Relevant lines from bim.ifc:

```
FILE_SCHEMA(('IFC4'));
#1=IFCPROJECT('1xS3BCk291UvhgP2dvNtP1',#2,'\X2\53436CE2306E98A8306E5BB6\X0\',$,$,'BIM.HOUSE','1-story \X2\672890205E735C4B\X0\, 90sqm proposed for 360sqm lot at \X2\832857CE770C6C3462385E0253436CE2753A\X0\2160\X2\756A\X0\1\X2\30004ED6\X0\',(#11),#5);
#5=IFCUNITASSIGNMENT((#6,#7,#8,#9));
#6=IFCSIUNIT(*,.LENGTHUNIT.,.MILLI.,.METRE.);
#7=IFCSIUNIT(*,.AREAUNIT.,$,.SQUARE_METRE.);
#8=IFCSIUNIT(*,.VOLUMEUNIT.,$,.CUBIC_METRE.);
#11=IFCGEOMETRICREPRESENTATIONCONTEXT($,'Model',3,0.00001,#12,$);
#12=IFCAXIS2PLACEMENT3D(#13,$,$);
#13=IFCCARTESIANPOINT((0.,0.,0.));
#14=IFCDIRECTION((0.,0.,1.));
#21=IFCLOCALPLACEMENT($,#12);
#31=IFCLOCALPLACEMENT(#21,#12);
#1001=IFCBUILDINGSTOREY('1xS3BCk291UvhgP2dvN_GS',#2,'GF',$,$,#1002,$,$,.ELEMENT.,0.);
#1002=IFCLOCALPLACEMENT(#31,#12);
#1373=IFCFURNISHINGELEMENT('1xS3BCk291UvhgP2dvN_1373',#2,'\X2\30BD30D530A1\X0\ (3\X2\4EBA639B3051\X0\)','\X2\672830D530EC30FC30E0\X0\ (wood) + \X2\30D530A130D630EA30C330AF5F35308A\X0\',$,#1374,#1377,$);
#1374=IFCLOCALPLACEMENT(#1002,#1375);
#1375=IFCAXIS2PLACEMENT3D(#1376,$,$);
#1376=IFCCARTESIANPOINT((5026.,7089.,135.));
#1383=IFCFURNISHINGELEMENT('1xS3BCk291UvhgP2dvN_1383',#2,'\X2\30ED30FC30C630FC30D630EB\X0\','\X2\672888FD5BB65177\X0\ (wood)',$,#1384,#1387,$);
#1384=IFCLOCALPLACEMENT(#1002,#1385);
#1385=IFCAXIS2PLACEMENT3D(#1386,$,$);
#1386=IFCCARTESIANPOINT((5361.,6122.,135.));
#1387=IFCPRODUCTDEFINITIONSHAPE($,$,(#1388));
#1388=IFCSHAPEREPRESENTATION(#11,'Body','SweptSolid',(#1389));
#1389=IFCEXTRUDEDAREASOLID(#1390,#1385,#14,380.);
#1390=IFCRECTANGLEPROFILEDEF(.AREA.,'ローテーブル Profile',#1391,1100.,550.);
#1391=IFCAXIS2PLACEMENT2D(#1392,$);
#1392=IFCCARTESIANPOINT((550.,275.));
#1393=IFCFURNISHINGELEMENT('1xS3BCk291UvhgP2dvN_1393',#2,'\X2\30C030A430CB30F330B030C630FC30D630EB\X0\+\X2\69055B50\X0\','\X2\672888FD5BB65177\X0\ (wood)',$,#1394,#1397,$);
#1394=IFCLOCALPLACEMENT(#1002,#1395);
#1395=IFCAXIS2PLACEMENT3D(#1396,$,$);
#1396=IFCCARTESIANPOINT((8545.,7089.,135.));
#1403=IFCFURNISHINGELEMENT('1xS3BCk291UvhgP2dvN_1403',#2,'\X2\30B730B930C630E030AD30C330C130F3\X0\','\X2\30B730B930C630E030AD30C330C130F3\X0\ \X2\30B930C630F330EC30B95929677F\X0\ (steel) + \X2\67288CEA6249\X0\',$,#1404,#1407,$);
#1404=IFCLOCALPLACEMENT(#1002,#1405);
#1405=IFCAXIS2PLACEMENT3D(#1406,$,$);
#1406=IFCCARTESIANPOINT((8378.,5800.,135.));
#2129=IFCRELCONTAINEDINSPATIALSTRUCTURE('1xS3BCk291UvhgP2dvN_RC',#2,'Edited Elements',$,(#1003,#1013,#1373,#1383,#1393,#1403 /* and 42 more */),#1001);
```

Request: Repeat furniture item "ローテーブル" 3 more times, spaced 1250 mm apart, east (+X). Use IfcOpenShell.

```python
import numpy as np
import ifcopenshell
import ifcopenshell.api.geometry
import ifcopenshell.api.root
import ifcopenshell.util.element
import ifcopenshell.util.placement

model = ifcopenshell.open("bim.ifc")


def reuse_history(source, copy):
    """copy_class also copies each property set's owner history, people and application; keep the originals."""
    for rel in copy.IsDefinedBy:
        if rel.is_a("IfcRelDefinesByProperties") and (history := rel.RelatingPropertyDefinition.OwnerHistory):
            rel.RelatingPropertyDefinition.OwnerHistory = source.OwnerHistory
            ifcopenshell.util.element.remove_deep2(model, history)


source = model.by_guid("1xS3BCk291UvhgP2dvN_1383")
base = ifcopenshell.util.placement.get_local_placement(source.ObjectPlacement)
step = np.array([1.0, 0.0, 0.0]) * 1250.0

for i in range(1, 4):
    copy = ifcopenshell.api.root.copy_class(model, product=source)
    copy.Representation = ifcopenshell.util.element.copy_deep(
        model, source.Representation, exclude=["IfcGeometricRepresentationContext", "IfcRepresentationMap"]
    )
    reuse_history(source, copy)
    matrix = base.copy()
    matrix[:3, 3] += i * step
    print("added at", matrix[:3, 3].round(3) + 0.0)
    ifcopenshell.api.geometry.edit_object_placement(model, product=copy, matrix=matrix, is_si=False)

model.write("bim-out.ifc")
```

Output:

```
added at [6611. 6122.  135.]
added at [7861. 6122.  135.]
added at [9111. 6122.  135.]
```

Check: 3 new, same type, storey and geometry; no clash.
